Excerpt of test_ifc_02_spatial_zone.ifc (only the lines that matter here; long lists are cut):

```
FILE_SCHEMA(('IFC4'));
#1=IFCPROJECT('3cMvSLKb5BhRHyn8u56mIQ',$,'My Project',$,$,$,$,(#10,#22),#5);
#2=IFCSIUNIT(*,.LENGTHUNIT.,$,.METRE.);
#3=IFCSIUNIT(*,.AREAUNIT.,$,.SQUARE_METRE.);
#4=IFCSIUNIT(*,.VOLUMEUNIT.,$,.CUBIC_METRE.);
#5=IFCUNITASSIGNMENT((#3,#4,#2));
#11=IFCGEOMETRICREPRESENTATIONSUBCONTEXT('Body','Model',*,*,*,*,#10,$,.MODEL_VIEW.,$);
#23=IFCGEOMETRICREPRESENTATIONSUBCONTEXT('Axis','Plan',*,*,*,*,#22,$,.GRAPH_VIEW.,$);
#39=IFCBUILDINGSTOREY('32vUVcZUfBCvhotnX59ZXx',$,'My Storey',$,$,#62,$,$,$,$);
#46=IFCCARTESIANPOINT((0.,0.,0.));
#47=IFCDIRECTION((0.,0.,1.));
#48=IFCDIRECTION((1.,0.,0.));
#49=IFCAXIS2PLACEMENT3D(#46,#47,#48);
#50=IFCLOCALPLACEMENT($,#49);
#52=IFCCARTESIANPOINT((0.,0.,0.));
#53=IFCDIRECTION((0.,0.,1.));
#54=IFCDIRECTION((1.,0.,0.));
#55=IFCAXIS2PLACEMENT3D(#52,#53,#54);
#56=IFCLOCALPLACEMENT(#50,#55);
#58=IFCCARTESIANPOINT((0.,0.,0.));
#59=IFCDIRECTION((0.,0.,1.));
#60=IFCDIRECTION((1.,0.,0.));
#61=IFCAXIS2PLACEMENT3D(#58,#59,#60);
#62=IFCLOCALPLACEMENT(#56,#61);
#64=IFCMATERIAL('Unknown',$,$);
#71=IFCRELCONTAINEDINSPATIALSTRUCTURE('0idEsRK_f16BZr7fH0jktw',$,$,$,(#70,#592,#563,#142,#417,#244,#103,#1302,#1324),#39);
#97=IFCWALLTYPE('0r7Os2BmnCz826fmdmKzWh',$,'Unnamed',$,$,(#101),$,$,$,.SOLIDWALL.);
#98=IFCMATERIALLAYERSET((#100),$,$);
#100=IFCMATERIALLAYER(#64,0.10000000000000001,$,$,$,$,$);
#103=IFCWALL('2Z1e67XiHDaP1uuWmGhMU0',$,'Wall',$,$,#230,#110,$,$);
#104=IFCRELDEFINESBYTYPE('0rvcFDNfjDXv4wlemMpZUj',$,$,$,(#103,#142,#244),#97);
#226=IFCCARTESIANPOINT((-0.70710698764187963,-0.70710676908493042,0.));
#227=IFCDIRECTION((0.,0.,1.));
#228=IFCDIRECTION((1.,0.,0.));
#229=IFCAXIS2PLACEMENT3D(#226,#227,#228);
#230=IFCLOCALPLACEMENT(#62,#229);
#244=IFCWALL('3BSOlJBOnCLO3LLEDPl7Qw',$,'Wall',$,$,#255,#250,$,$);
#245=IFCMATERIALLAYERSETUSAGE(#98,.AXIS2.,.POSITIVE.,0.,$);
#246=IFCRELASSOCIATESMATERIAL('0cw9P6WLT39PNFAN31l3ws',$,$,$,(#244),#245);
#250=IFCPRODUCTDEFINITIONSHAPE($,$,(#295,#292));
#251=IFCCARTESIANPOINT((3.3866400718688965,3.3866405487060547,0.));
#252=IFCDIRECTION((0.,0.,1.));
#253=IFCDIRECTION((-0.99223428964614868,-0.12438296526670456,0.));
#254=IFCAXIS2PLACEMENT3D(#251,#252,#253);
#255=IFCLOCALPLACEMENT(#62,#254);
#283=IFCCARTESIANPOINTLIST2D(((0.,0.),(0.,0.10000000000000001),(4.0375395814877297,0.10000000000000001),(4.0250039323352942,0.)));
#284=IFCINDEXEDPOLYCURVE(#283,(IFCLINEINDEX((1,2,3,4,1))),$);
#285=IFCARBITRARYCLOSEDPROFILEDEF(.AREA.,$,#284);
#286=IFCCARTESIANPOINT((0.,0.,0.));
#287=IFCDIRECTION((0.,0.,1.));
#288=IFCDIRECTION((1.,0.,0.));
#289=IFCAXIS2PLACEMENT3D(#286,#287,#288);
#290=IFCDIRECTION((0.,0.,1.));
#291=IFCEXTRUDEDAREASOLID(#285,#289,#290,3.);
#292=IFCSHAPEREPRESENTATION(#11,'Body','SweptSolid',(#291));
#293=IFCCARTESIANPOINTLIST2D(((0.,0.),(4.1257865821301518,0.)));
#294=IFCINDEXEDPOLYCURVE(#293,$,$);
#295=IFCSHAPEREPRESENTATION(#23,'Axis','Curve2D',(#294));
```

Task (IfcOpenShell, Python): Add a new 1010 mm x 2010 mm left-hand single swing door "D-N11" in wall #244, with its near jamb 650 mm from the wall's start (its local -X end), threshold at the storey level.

```python
import numpy as np
import ifcopenshell
import ifcopenshell.api.feature
import ifcopenshell.api.geometry
import ifcopenshell.api.root
import ifcopenshell.api.spatial
import ifcopenshell.geom
import ifcopenshell.util.element
import ifcopenshell.util.placement
import ifcopenshell.util.representation
import ifcopenshell.util.shape
import ifcopenshell.util.unit

model = ifcopenshell.open("test_ifc_02_spatial_zone.ifc")
unit_scale = ifcopenshell.util.unit.calculate_unit_scale(model)
settings = ifcopenshell.geom.settings()


def volume(element):
    """Net volume in cubic metres, openings subtracted."""
    shape = ifcopenshell.geom.create_shape(settings, element)
    return ifcopenshell.util.shape.get_volume(shape.geometry)


wall = model.by_guid("3BSOlJBOnCLO3LLEDPl7Qw")
storey = ifcopenshell.util.element.get_container(wall, ifc_class="IfcBuildingStorey")
context = ifcopenshell.util.representation.get_context(model, "Model", "Body", "MODEL_VIEW")
before = volume(wall)

width, height, from_end, sill = 1.01, 2.01, 0.65, 0.0  # metres

# The wall runs along its own X axis, and the end named is its -X end.
wall_shape = ifcopenshell.geom.create_shape(settings, wall)
x, y, z = ifcopenshell.util.shape.get_vertices(wall_shape.geometry).T
start = x.min() + from_end
face, thickness = float(y.min()), float(y.max() - y.min())
wall_matrix = ifcopenshell.util.placement.get_local_placement(wall.ObjectPlacement)
level = ifcopenshell.util.placement.get_local_placement(storey.ObjectPlacement)[2, 3]


def in_wall(x, y):
    """Placement at x, y metres in the wall's axes, at sill height."""
    matrix = wall_matrix.copy()
    matrix[:, 3] = wall_matrix @ np.array([x / unit_scale, y / unit_scale, 0.0, 1.0])
    matrix[2, 3] = level + sill / unit_scale
    return matrix


# Opening: a box that overshoots both wall faces by 50 mm.
opening = ifcopenshell.api.root.create_entity(model, ifc_class="IfcOpeningElement", predefined_type="OPENING")
box = ifcopenshell.api.geometry.add_wall_representation(
    model, context=context, length=width, height=height, thickness=thickness + 0.1
)
ifcopenshell.api.geometry.assign_representation(model, product=opening, representation=box)
ifcopenshell.api.geometry.edit_object_placement(model, product=opening, matrix=in_wall(start, face - 0.05), is_si=False)
ifcopenshell.api.feature.add_feature(model, feature=opening, element=wall)

door = ifcopenshell.api.root.create_entity(model, ifc_class="IfcDoor", name="D-N11", predefined_type="DOOR")
door.OverallWidth, door.OverallHeight = width / unit_scale, height / unit_scale
door.OperationType = "SINGLE_SWING_LEFT"
body = ifcopenshell.api.geometry.add_door_representation(
    model,
    context=context,
    overall_width=door.OverallWidth,
    overall_height=door.OverallHeight,
    operation_type="SINGLE_SWING_LEFT",
    lining_properties={"LiningDepth": thickness / unit_scale, "ThresholdDepth": thickness / unit_scale},
)
ifcopenshell.api.geometry.assign_representation(model, product=door, representation=body)
ifcopenshell.api.spatial.assign_container(model, products=[door], relating_structure=storey)
ifcopenshell.api.feature.add_filling(model, opening=opening, element=door)

# The lining spans the wall, so the door starts at the wall face.
ifcopenshell.api.geometry.edit_object_placement(model, product=door, matrix=in_wall(start, face), is_si=False)

after = volume(wall)

print(f"wall volume {before:.3f} -> {after:.3f} m3")

model.write("test_ifc_02_spatial_zone_rev.ifc")
```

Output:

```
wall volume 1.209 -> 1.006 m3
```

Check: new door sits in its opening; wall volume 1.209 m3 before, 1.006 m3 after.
